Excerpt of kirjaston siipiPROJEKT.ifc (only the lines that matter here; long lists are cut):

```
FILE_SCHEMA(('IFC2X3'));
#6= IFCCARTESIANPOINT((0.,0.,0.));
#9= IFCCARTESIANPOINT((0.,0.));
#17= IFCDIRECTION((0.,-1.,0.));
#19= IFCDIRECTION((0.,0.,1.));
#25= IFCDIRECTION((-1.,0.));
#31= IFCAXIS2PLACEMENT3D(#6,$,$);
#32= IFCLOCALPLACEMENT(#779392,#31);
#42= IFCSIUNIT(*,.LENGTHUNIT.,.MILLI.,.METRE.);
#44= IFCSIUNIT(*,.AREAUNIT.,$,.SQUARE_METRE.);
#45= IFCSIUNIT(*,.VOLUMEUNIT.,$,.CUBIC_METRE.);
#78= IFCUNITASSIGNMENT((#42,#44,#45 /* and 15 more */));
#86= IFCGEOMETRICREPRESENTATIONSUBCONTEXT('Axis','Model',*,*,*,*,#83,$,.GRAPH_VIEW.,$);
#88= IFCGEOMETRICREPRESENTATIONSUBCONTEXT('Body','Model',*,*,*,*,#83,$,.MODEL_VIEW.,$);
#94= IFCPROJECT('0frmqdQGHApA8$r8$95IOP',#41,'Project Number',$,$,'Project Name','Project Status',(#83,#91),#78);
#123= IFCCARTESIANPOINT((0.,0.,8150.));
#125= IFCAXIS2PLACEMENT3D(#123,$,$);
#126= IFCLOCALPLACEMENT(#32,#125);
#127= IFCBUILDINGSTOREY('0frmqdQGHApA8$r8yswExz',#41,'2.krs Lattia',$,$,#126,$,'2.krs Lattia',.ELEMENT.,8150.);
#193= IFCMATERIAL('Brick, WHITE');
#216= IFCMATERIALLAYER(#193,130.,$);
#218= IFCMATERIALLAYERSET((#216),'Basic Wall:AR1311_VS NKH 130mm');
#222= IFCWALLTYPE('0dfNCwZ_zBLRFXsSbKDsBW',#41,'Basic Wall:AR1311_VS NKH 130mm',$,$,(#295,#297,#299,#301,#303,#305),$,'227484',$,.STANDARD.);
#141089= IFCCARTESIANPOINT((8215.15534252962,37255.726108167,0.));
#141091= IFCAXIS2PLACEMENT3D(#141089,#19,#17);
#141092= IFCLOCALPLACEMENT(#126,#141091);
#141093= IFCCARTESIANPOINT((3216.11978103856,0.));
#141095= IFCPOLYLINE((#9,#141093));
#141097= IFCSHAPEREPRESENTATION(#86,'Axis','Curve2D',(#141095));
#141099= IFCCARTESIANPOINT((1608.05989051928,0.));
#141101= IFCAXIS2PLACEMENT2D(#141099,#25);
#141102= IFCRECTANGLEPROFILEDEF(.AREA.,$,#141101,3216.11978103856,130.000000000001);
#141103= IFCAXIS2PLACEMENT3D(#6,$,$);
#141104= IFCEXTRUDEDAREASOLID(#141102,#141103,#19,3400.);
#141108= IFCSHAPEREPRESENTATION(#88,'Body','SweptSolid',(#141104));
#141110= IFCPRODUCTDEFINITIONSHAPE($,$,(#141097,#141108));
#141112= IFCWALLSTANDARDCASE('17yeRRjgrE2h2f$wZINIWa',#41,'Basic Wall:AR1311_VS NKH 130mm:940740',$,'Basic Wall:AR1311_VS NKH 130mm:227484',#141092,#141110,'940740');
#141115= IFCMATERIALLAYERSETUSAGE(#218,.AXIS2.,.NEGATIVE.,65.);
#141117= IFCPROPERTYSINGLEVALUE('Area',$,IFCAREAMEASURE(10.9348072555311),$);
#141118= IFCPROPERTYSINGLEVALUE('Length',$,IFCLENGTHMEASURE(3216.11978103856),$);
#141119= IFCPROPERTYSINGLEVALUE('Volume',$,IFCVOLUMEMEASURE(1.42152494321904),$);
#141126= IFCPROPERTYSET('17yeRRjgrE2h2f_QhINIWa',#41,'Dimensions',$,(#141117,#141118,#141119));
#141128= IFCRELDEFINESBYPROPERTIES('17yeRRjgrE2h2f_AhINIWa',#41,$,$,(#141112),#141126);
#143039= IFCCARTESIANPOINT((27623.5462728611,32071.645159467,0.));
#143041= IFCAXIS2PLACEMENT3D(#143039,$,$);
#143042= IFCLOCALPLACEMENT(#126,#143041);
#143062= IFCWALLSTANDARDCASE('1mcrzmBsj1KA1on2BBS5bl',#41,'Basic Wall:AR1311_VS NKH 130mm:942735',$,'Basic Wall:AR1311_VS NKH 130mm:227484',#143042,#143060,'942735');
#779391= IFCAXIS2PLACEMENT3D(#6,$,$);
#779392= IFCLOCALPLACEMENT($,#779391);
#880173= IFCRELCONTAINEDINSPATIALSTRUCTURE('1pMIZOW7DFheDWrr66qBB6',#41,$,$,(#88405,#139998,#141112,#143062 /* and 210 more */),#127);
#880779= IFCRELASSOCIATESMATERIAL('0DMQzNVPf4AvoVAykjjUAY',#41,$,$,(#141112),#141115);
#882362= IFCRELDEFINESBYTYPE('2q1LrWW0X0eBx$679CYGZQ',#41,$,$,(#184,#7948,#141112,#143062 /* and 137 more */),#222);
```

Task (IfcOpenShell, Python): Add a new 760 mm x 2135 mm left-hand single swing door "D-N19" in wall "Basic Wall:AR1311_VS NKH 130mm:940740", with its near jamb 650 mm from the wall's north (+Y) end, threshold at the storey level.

```python
import numpy as np
import ifcopenshell
import ifcopenshell.api.feature
import ifcopenshell.api.geometry
import ifcopenshell.api.pset
import ifcopenshell.api.root
import ifcopenshell.api.spatial
import ifcopenshell.api.type
import ifcopenshell.geom
import ifcopenshell.util.element
import ifcopenshell.util.placement
import ifcopenshell.util.representation
import ifcopenshell.util.shape
import ifcopenshell.util.unit

model = ifcopenshell.open("kirjaston siipiPROJEKT.ifc")
unit_scale = ifcopenshell.util.unit.calculate_unit_scale(model)
area_scale = ifcopenshell.util.unit.calculate_unit_scale(model, "AREAUNIT")
volume_scale = ifcopenshell.util.unit.calculate_unit_scale(model, "VOLUMEUNIT")
settings = ifcopenshell.geom.settings()


def volume(element):
    """Net volume in cubic metres, openings subtracted."""
    shape = ifcopenshell.geom.create_shape(settings, element)
    return ifcopenshell.util.shape.get_volume(shape.geometry)


wall = model.by_guid("17yeRRjgrE2h2f$wZINIWa")
storey = ifcopenshell.util.element.get_container(wall, ifc_class="IfcBuildingStorey")
context = ifcopenshell.util.representation.get_context(model, "Model", "Body", "MODEL_VIEW")
before = volume(wall)

width, height, from_end, sill = 0.76, 2.135, 0.65, 0.0  # metres

# The wall runs along its own X axis, and the end named is its -X end.
wall_shape = ifcopenshell.geom.create_shape(settings, wall)
x, y, z = ifcopenshell.util.shape.get_vertices(wall_shape.geometry).T
start = x.min() + from_end
face, thickness = float(y.min()), float(y.max() - y.min())
wall_matrix = ifcopenshell.util.placement.get_local_placement(wall.ObjectPlacement)
level = ifcopenshell.util.placement.get_local_placement(storey.ObjectPlacement)[2, 3]


def in_wall(x, y):
    """Placement at x, y metres in the wall's axes, at sill height."""
    matrix = wall_matrix.copy()
    matrix[:, 3] = wall_matrix @ np.array([x / unit_scale, y / unit_scale, 0.0, 1.0])
    matrix[2, 3] = level + sill / unit_scale
    return matrix


# Opening: a box that overshoots both wall faces by 50 mm.
opening = ifcopenshell.api.root.create_entity(model, ifc_class="IfcOpeningElement")
box = ifcopenshell.api.geometry.add_wall_representation(
    model, context=context, length=width, height=height, thickness=thickness + 0.1
)
ifcopenshell.api.geometry.assign_representation(model, product=opening, representation=box)
ifcopenshell.api.geometry.edit_object_placement(model, product=opening, matrix=in_wall(start, face - 0.05), is_si=False)
ifcopenshell.api.feature.add_feature(model, feature=opening, element=wall)

door = ifcopenshell.api.root.create_entity(model, ifc_class="IfcDoor", name="D-N19")
door.OverallWidth, door.OverallHeight = width / unit_scale, height / unit_scale
body = ifcopenshell.api.geometry.add_door_representation(
    model,
    context=context,
    overall_width=door.OverallWidth,
    overall_height=door.OverallHeight,
    operation_type="SINGLE_SWING_LEFT",
    lining_properties={"LiningDepth": thickness / unit_scale, "ThresholdDepth": thickness / unit_scale},
)
ifcopenshell.api.geometry.assign_representation(model, product=door, representation=body)
ifcopenshell.api.spatial.assign_container(model, products=[door], relating_structure=storey)
fills = ifcopenshell.api.feature.add_filling(model, opening=opening, element=door)
fills.OwnerHistory = door.OwnerHistory  # required in IFC2X3

# IFC2X3 keeps the operation on the door style.
style = ifcopenshell.api.root.create_entity(model, ifc_class="IfcDoorStyle", name="D-N19")
style.OperationType, style.ConstructionType = "SINGLE_SWING_LEFT", "NOTDEFINED"
style.ParameterTakesPrecedence = style.Sizeable = False
ifcopenshell.api.type.assign_type(model, related_objects=[door], relating_type=style)

# The lining spans the wall, so the door starts at the wall face.
ifcopenshell.api.geometry.edit_object_placement(model, product=door, matrix=in_wall(start, face), is_si=False)

after = volume(wall)

# Update the wall's stored quantities.
pset = model.by_id(ifcopenshell.util.element.get_pset(wall, "Dimensions", should_inherit=False)["id"])
ifcopenshell.api.pset.edit_pset(model, pset=pset, properties={
    "Area": model.create_entity("IfcAreaMeasure", after / thickness / area_scale),
    "Volume": model.create_entity("IfcVolumeMeasure", after / volume_scale),
})

print(f"wall volume {before:.3f} -> {after:.3f} m3")

model.write("kirjaston siipiPROJEKT_edited.ifc")
```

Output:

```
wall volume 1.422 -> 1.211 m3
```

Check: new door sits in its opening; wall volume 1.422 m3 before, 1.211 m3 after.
